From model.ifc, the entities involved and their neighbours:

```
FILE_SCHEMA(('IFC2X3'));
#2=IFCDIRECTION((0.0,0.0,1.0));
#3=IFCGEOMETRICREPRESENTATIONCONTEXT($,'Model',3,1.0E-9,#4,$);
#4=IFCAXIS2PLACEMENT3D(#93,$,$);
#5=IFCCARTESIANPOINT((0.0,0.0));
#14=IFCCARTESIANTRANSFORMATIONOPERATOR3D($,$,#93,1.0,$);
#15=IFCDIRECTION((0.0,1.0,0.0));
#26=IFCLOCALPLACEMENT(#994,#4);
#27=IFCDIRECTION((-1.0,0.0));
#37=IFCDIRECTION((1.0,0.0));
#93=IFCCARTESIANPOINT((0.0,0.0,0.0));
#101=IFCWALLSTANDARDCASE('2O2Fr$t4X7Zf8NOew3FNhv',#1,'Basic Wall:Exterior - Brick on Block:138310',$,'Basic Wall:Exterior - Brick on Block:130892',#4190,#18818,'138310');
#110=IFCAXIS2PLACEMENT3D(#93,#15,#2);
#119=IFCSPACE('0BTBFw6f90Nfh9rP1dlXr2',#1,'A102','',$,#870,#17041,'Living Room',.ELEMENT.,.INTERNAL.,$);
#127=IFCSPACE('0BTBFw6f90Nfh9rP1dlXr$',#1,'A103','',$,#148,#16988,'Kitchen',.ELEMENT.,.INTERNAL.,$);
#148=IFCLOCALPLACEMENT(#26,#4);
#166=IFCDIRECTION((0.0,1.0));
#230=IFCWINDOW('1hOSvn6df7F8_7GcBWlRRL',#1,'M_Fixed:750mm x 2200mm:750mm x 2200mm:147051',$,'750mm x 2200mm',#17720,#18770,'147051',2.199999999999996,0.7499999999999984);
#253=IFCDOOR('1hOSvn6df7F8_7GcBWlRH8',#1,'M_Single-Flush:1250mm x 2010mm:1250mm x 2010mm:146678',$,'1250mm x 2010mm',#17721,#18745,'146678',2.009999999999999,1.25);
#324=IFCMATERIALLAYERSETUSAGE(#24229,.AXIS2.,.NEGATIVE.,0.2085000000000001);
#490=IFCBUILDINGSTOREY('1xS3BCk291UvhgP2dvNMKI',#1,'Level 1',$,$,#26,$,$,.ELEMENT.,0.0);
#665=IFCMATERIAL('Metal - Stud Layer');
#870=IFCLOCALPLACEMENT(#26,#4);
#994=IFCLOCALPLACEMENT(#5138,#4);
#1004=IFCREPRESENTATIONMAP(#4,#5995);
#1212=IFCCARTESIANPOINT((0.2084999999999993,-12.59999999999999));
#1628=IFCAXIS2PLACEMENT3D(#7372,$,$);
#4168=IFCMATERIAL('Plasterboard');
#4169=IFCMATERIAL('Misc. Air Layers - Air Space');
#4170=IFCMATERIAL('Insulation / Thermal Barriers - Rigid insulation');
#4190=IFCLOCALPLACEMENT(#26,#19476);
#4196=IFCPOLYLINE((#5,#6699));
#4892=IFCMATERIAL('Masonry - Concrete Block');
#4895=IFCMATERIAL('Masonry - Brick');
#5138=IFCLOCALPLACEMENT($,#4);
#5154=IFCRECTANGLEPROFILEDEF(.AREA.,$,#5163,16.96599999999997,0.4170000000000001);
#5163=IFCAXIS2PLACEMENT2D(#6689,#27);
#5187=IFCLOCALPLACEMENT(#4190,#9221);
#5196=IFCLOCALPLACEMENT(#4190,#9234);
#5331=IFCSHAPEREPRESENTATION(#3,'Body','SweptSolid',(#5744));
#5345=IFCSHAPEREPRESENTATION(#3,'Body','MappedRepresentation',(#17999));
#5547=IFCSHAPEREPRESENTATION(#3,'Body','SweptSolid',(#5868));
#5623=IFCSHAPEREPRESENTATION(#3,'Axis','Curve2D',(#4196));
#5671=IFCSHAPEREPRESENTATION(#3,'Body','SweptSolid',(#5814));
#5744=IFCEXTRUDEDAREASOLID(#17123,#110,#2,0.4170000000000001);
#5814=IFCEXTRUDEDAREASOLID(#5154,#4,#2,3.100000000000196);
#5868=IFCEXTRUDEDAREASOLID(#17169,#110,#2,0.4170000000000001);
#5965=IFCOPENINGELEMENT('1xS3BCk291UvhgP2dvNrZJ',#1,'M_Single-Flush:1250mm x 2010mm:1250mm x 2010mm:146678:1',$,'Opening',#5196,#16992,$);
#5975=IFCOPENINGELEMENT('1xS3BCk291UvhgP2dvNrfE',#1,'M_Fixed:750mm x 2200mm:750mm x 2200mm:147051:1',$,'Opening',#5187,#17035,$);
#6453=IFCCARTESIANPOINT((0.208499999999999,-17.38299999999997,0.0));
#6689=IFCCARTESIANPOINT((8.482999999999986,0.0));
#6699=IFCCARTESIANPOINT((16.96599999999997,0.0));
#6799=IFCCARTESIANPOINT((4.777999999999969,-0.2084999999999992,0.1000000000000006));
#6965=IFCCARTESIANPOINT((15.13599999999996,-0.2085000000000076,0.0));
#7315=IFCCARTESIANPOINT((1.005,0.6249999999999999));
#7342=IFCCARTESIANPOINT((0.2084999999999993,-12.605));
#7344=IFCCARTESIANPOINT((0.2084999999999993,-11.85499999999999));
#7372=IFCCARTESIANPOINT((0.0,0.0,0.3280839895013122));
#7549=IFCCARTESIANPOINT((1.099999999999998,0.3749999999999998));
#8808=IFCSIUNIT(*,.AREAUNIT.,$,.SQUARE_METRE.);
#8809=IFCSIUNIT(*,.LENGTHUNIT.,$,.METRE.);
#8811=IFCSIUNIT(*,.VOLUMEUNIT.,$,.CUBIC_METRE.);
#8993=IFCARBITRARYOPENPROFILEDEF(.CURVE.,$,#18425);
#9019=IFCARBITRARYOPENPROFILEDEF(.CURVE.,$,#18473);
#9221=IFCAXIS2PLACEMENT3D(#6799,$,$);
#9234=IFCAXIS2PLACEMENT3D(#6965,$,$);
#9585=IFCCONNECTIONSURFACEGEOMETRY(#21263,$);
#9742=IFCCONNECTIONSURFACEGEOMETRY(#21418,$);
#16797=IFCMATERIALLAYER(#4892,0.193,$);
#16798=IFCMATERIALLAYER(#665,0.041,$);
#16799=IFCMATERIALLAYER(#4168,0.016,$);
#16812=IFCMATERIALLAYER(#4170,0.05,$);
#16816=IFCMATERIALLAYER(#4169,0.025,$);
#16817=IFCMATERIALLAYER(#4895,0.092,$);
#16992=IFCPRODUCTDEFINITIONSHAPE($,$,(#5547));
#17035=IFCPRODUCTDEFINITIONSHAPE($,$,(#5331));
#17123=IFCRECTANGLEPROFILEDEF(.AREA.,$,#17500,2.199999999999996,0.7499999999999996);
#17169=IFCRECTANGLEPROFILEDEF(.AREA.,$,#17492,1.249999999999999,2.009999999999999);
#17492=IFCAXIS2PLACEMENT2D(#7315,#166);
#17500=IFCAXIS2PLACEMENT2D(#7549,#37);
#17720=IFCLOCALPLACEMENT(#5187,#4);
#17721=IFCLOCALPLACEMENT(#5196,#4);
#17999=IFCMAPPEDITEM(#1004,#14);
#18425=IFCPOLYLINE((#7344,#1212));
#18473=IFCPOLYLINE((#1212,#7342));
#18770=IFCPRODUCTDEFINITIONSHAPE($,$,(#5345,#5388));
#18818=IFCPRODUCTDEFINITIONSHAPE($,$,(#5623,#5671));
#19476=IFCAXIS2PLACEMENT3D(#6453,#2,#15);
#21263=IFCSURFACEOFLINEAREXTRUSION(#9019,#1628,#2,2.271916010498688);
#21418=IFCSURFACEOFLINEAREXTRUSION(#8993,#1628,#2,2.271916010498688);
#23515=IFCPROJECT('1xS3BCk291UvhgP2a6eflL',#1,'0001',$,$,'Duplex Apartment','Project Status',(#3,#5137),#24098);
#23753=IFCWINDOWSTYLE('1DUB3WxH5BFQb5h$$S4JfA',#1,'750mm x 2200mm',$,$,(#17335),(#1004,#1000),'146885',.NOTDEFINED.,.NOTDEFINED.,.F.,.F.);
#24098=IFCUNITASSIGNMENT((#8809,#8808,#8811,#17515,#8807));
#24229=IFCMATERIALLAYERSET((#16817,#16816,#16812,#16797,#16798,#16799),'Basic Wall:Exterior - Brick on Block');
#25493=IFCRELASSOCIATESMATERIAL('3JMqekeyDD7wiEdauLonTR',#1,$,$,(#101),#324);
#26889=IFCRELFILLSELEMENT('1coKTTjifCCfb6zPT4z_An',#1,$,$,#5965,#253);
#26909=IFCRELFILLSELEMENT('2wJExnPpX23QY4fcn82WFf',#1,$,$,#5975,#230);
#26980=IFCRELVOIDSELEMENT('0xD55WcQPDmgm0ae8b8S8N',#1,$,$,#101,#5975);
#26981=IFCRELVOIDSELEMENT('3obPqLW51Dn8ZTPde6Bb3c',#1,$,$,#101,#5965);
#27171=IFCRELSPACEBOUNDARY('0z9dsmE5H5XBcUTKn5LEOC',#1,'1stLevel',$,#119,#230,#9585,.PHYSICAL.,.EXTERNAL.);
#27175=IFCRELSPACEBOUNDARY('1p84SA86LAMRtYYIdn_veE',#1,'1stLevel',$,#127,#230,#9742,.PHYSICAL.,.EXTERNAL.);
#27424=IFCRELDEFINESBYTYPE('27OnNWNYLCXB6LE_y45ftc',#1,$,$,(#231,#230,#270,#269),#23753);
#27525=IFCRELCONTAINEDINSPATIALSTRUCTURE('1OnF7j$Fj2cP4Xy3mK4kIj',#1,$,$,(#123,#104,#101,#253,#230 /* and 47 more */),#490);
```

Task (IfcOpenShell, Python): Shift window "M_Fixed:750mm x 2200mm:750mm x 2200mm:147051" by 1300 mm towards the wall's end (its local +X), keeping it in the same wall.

```python
import numpy as np
import ifcopenshell
import ifcopenshell.api.geometry
import ifcopenshell.util.placement

model = ifcopenshell.open("model.ifc")

window = model.by_guid("1hOSvn6df7F8_7GcBWlRRL")
opening = window.FillsVoids[0].RelatingOpeningElement
wall = opening.VoidsElements[0].RelatingBuildingElement

wall_matrix = ifcopenshell.util.placement.get_local_placement(wall.ObjectPlacement)
shift = wall_matrix[:3, 0] * 1.3
before = ifcopenshell.util.placement.get_local_placement(window.ObjectPlacement)[:3, 3].copy()

# The window is placed relative to its opening, so it follows when the opening moves.
matrix = ifcopenshell.util.placement.get_local_placement(opening.ObjectPlacement)
matrix[:3, 3] += shift
ifcopenshell.api.geometry.edit_object_placement(
    model, product=opening, matrix=matrix, is_si=False, should_transform_children=True
)

# Space boundary surfaces are stored in each space's coordinates; move them too.
for rel in window.ProvidesBoundaries:
    if not rel.ConnectionGeometry:
        continue
    surface = rel.ConnectionGeometry.SurfaceOnRelatingElement
    space_matrix = ifcopenshell.util.placement.get_local_placement(rel.RelatingSpace.ObjectPlacement)
    point = np.array(surface.Position.Location.Coordinates) + space_matrix[:3, :3].T @ shift
    surface.Position = model.createIfcAxis2Placement3D(
        model.createIfcCartesianPoint(point.tolist()), surface.Position.Axis, surface.Position.RefDirection
    )

after = ifcopenshell.util.placement.get_local_placement(window.ObjectPlacement)[:3, 3]
print("window moved by", (after - before).round(3) + 0.0)

model.write("model_updated.ifc")
```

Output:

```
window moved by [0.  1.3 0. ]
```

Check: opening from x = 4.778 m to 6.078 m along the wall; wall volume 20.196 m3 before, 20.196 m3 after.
